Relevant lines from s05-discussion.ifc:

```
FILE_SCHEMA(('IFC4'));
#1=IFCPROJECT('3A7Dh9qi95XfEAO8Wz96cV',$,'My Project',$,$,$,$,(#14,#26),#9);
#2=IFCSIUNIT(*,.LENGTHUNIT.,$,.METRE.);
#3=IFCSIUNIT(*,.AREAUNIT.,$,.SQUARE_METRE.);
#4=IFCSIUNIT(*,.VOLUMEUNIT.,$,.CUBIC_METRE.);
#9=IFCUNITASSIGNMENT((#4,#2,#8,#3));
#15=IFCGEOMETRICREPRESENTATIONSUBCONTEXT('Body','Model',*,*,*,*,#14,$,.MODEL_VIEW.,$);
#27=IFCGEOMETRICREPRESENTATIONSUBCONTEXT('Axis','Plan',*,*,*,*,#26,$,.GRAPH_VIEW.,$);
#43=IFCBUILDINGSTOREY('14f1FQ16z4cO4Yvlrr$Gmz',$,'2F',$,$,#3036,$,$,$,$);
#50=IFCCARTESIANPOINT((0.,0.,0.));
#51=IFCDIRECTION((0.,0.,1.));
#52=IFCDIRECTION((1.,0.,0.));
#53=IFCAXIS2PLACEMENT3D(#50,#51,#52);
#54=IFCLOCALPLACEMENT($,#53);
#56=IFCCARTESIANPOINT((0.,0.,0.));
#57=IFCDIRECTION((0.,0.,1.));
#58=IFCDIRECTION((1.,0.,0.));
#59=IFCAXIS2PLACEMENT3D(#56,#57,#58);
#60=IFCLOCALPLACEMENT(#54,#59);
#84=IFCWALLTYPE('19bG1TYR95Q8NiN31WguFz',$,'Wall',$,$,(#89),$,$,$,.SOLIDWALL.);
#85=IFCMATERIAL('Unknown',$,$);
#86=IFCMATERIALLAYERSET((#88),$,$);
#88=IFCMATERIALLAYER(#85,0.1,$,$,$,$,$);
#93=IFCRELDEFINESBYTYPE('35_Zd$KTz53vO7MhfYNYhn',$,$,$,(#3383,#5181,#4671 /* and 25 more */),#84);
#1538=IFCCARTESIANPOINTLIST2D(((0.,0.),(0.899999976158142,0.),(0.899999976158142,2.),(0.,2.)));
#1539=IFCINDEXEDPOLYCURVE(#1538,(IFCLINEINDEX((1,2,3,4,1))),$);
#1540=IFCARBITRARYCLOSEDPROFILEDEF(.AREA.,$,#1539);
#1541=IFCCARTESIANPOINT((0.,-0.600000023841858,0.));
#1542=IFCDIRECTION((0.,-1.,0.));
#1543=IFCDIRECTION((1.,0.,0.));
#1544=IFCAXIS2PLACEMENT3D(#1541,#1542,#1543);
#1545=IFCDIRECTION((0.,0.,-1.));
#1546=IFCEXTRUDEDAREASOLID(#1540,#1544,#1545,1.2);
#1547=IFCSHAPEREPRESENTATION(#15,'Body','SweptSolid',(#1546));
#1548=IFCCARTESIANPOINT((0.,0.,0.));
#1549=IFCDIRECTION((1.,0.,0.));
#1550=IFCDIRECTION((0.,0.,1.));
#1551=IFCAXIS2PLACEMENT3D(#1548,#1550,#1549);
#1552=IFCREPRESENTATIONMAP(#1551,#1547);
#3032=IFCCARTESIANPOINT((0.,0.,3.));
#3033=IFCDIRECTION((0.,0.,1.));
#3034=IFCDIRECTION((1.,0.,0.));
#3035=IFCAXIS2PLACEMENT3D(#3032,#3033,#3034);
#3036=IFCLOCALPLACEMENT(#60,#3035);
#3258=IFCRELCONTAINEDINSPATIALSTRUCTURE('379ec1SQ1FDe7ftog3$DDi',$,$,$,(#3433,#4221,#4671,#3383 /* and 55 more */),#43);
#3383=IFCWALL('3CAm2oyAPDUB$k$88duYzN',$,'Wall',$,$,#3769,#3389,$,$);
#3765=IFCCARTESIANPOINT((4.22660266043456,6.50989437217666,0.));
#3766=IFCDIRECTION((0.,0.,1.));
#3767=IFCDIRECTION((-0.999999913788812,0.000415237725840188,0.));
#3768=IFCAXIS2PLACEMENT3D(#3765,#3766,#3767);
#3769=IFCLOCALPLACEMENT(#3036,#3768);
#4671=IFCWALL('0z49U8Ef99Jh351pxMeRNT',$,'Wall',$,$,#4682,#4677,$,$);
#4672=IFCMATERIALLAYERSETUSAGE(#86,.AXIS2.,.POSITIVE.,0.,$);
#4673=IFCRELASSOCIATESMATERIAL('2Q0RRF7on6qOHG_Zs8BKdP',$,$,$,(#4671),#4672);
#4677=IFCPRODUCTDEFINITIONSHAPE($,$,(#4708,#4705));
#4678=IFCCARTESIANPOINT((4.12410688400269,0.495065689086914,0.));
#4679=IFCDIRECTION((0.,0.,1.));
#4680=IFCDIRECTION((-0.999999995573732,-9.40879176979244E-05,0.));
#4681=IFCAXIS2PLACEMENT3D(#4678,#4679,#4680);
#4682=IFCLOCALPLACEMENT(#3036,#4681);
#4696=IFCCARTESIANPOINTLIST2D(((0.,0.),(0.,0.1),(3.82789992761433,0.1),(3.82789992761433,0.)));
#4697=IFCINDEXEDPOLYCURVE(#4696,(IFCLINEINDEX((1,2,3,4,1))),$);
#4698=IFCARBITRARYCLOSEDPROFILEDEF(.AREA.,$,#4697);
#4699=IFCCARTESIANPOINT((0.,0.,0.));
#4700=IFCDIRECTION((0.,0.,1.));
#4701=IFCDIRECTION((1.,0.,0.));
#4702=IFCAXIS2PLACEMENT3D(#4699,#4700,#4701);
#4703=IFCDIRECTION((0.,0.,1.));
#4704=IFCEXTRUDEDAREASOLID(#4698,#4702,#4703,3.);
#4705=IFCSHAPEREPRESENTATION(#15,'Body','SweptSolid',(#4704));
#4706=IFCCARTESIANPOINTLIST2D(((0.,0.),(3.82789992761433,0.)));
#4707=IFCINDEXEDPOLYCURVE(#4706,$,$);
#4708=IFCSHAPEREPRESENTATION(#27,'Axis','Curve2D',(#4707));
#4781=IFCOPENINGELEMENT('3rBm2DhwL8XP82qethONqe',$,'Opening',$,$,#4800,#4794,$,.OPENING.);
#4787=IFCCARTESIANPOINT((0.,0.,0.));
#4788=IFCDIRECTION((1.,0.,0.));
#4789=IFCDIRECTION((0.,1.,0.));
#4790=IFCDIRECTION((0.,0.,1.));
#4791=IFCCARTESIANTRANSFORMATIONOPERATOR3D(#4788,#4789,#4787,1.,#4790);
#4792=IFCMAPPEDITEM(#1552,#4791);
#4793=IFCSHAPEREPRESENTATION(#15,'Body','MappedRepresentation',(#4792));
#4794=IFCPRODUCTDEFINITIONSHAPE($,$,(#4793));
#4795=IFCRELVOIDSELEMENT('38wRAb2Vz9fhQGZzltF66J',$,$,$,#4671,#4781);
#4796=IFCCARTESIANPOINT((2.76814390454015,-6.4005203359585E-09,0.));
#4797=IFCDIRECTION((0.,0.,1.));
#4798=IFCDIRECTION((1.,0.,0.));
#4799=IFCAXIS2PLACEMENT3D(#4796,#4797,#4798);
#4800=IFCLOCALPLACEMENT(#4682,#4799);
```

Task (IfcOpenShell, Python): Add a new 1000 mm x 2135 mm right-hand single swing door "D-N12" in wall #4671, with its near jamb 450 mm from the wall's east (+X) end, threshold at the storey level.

```python
import numpy as np
import ifcopenshell
import ifcopenshell.api.feature
import ifcopenshell.api.geometry
import ifcopenshell.api.root
import ifcopenshell.api.spatial
import ifcopenshell.geom
import ifcopenshell.util.element
import ifcopenshell.util.placement
import ifcopenshell.util.representation
import ifcopenshell.util.shape
import ifcopenshell.util.unit

model = ifcopenshell.open("s05-discussion.ifc")
unit_scale = ifcopenshell.util.unit.calculate_unit_scale(model)
settings = ifcopenshell.geom.settings()


def volume(element):
    """Net volume in cubic metres, openings subtracted."""
    shape = ifcopenshell.geom.create_shape(settings, element)
    return ifcopenshell.util.shape.get_volume(shape.geometry)


wall = model.by_guid("0z49U8Ef99Jh351pxMeRNT")
storey = ifcopenshell.util.element.get_container(wall, ifc_class="IfcBuildingStorey")
context = ifcopenshell.util.representation.get_context(model, "Model", "Body", "MODEL_VIEW")
before = volume(wall)

width, height, from_end, sill = 1, 2.135, 0.45, 0.0  # metres

# The wall runs along its own X axis, and the end named is its -X end.
wall_shape = ifcopenshell.geom.create_shape(settings, wall)
x, y, z = ifcopenshell.util.shape.get_vertices(wall_shape.geometry).T
start = x.min() + from_end
face, thickness = float(y.min()), float(y.max() - y.min())
wall_matrix = ifcopenshell.util.placement.get_local_placement(wall.ObjectPlacement)
level = ifcopenshell.util.placement.get_local_placement(storey.ObjectPlacement)[2, 3]


def in_wall(x, y):
    """Placement at x, y metres in the wall's axes, at sill height."""
    matrix = wall_matrix.copy()
    matrix[:, 3] = wall_matrix @ np.array([x / unit_scale, y / unit_scale, 0.0, 1.0])
    matrix[2, 3] = level + sill / unit_scale
    return matrix


# Opening: a box that overshoots both wall faces by 50 mm.
opening = ifcopenshell.api.root.create_entity(model, ifc_class="IfcOpeningElement", predefined_type="OPENING")
box = ifcopenshell.api.geometry.add_wall_representation(
    model, context=context, length=width, height=height, thickness=thickness + 0.1
)
ifcopenshell.api.geometry.assign_representation(model, product=opening, representation=box)
ifcopenshell.api.geometry.edit_object_placement(model, product=opening, matrix=in_wall(start, face - 0.05), is_si=False)
ifcopenshell.api.feature.add_feature(model, feature=opening, element=wall)

door = ifcopenshell.api.root.create_entity(model, ifc_class="IfcDoor", name="D-N12", predefined_type="DOOR")
door.OverallWidth, door.OverallHeight = width / unit_scale, height / unit_scale
door.OperationType = "SINGLE_SWING_RIGHT"
body = ifcopenshell.api.geometry.add_door_representation(
    model,
    context=context,
    overall_width=door.OverallWidth,
    overall_height=door.OverallHeight,
    operation_type="SINGLE_SWING_RIGHT",
    lining_properties={"LiningDepth": thickness / unit_scale, "ThresholdDepth": thickness / unit_scale},
)
ifcopenshell.api.geometry.assign_representation(model, product=door, representation=body)
ifcopenshell.api.spatial.assign_container(model, products=[door], relating_structure=storey)
ifcopenshell.api.feature.add_filling(model, opening=opening, element=door)

# The lining spans the wall, so the door starts at the wall face.
ifcopenshell.api.geometry.edit_object_placement(model, product=door, matrix=in_wall(start, face), is_si=False)

after = volume(wall)

print(f"wall volume {before:.3f} -> {after:.3f} m3")

model.write("s05-discussion_rev.ifc")
```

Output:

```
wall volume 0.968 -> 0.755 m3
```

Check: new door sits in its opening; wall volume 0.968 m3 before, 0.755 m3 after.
